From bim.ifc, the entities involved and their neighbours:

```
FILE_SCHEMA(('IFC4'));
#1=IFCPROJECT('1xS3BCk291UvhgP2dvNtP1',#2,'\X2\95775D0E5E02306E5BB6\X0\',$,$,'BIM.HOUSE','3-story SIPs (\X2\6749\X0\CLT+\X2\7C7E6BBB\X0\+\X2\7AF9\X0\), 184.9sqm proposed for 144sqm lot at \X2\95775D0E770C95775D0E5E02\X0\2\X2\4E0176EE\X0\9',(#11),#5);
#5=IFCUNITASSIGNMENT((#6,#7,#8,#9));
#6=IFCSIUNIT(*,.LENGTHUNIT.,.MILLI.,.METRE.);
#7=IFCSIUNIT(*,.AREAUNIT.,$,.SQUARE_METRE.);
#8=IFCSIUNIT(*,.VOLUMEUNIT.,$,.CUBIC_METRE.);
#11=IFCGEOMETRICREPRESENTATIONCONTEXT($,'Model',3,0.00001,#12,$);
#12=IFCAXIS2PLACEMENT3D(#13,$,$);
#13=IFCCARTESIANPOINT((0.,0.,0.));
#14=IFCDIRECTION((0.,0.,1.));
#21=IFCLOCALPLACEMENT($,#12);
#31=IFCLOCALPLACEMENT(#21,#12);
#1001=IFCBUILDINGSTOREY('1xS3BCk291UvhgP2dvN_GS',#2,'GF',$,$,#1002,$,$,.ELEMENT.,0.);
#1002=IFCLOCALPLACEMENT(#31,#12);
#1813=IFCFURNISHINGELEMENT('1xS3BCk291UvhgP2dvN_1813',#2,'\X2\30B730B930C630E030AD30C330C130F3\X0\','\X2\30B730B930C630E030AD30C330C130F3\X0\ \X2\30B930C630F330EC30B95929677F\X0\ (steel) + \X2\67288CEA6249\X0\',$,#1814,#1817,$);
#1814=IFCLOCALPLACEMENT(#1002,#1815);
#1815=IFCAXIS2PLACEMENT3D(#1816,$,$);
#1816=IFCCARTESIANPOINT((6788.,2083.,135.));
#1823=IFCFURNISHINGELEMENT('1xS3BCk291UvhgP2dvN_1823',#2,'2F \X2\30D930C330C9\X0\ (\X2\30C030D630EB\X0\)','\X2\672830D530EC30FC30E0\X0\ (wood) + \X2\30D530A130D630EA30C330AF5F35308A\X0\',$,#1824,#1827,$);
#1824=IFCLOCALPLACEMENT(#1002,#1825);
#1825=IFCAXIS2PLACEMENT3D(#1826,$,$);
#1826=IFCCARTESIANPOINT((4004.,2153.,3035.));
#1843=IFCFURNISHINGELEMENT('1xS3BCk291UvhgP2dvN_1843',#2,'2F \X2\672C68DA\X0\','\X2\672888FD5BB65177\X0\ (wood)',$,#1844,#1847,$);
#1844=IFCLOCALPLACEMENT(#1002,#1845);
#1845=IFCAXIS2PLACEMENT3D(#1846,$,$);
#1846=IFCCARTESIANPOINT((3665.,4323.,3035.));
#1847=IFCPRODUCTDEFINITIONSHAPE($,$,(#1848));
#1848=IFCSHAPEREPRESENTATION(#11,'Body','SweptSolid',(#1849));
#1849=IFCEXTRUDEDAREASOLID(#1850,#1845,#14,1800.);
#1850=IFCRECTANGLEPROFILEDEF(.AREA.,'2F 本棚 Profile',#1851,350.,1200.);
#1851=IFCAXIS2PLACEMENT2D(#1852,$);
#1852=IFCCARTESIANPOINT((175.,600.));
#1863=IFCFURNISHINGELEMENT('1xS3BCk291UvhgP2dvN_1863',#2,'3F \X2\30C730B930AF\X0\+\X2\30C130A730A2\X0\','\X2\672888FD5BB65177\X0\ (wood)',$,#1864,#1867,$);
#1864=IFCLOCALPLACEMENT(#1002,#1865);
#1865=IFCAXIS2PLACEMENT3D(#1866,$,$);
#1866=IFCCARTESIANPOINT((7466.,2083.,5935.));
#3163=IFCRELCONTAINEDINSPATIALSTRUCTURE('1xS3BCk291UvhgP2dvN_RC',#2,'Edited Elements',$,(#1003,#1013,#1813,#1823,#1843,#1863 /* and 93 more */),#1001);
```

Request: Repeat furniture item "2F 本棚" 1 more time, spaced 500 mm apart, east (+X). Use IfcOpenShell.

```python
import numpy as np
import ifcopenshell
import ifcopenshell.api.geometry
import ifcopenshell.api.root
import ifcopenshell.util.element
import ifcopenshell.util.placement

model = ifcopenshell.open("bim.ifc")


def reuse_history(source, copy):
    """copy_class also copies each property set's owner history, people and application; keep the originals."""
    for rel in copy.IsDefinedBy:
        if rel.is_a("IfcRelDefinesByProperties") and (history := rel.RelatingPropertyDefinition.OwnerHistory):
            rel.RelatingPropertyDefinition.OwnerHistory = source.OwnerHistory
            ifcopenshell.util.element.remove_deep2(model, history)


source = model.by_guid("1xS3BCk291UvhgP2dvN_1843")
base = ifcopenshell.util.placement.get_local_placement(source.ObjectPlacement)
step = np.array([1.0, 0.0, 0.0]) * 500.0

for i in range(1, 2):
    copy = ifcopenshell.api.root.copy_class(model, product=source)
    copy.Representation = ifcopenshell.util.element.copy_deep(
        model, source.Representation, exclude=["IfcGeometricRepresentationContext", "IfcRepresentationMap"]
    )
    reuse_history(source, copy)
    matrix = base.copy()
    matrix[:3, 3] += i * step
    print("added at", matrix[:3, 3].round(3) + 0.0)
    ifcopenshell.api.geometry.edit_object_placement(model, product=copy, matrix=matrix, is_si=False)

model.write("bim_edited.ifc")
```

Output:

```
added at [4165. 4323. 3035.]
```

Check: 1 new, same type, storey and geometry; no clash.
